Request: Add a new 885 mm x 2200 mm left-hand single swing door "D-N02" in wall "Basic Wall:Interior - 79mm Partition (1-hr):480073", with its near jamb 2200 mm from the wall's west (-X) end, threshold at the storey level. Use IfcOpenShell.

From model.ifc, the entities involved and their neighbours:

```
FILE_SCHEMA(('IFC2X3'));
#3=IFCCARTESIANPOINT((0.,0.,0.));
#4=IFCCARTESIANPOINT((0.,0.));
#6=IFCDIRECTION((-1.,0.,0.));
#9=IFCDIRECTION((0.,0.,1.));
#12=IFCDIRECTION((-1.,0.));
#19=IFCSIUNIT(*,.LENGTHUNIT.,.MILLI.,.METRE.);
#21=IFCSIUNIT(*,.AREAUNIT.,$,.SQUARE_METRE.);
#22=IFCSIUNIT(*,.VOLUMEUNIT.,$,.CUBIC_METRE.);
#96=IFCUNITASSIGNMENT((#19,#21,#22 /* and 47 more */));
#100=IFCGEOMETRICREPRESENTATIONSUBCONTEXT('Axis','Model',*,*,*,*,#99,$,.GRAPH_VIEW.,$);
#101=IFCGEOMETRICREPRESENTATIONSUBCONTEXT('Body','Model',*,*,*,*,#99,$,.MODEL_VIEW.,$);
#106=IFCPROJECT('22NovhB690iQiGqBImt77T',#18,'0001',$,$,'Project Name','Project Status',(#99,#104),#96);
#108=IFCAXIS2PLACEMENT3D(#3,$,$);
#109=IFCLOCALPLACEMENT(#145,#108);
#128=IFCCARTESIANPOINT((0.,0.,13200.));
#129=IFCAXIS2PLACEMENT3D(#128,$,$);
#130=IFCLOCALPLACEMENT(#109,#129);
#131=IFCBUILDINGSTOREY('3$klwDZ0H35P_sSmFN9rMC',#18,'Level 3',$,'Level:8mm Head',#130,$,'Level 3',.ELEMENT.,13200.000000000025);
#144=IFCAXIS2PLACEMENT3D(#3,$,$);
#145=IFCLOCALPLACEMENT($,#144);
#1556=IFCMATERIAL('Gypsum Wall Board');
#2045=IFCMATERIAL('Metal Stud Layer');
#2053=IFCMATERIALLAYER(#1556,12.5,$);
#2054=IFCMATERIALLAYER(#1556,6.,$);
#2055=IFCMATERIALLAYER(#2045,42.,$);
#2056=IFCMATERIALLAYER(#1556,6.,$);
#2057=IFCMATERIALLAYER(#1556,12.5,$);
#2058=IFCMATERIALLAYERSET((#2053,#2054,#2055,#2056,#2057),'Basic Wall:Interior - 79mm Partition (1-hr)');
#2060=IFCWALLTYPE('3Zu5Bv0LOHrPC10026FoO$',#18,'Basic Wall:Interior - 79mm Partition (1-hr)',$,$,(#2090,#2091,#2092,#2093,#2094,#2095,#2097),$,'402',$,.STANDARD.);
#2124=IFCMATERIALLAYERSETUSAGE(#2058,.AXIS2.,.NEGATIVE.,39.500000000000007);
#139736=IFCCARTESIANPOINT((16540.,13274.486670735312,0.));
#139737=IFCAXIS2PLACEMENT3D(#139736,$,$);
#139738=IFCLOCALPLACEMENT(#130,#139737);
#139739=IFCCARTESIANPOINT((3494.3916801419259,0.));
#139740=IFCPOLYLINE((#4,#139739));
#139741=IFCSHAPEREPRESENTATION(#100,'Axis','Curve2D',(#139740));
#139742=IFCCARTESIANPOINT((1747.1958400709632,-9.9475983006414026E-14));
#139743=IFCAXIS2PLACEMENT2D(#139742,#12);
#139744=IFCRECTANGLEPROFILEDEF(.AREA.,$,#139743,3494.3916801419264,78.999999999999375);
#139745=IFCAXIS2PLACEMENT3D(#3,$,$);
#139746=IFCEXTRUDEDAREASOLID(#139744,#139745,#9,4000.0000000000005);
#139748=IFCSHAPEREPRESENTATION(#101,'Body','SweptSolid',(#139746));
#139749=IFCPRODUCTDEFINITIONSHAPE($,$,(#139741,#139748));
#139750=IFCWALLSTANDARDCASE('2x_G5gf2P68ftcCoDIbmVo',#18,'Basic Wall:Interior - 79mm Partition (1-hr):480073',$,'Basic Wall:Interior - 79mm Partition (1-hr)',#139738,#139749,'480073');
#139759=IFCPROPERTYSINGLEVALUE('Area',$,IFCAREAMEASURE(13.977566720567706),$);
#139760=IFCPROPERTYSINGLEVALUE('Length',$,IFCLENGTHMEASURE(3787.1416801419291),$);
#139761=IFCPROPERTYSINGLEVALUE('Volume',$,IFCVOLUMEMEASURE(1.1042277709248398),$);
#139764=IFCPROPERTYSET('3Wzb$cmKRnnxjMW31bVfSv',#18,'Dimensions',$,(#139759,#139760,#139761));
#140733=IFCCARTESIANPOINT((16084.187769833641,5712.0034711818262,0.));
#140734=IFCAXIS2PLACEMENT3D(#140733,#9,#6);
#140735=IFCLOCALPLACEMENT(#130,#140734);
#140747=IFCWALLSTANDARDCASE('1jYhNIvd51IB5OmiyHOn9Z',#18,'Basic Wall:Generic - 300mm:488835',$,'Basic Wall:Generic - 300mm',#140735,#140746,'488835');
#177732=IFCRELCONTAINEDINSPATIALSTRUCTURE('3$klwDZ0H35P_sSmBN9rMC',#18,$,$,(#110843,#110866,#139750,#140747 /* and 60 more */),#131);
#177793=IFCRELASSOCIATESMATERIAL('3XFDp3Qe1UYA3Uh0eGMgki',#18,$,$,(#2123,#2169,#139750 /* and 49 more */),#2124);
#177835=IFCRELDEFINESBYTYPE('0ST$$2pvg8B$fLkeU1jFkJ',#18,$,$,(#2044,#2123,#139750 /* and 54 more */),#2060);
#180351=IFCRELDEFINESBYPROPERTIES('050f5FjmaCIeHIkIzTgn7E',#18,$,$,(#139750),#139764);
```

```python
import numpy as np
import ifcopenshell
import ifcopenshell.api.feature
import ifcopenshell.api.geometry
import ifcopenshell.api.pset
import ifcopenshell.api.root
import ifcopenshell.api.spatial
import ifcopenshell.api.type
import ifcopenshell.geom
import ifcopenshell.util.element
import ifcopenshell.util.placement
import ifcopenshell.util.representation
import ifcopenshell.util.shape
import ifcopenshell.util.unit

model = ifcopenshell.open("model.ifc")
unit_scale = ifcopenshell.util.unit.calculate_unit_scale(model)
area_scale = ifcopenshell.util.unit.calculate_unit_scale(model, "AREAUNIT")
volume_scale = ifcopenshell.util.unit.calculate_unit_scale(model, "VOLUMEUNIT")
settings = ifcopenshell.geom.settings()


def volume(element):
    """Net volume in cubic metres, openings subtracted."""
    shape = ifcopenshell.geom.create_shape(settings, element)
    return ifcopenshell.util.shape.get_volume(shape.geometry)


wall = model.by_id(139750)
storey = ifcopenshell.util.element.get_container(wall, ifc_class="IfcBuildingStorey")
context = ifcopenshell.util.representation.get_context(model, "Model", "Body", "MODEL_VIEW")
before = volume(wall)

width, height, from_end, sill = 0.885, 2.2, 2.2, 0.0  # metres

# The wall runs along its own X axis, and the end named is its -X end.
wall_shape = ifcopenshell.geom.create_shape(settings, wall)
x, y, z = ifcopenshell.util.shape.get_vertices(wall_shape.geometry).T
start = x.min() + from_end
face, thickness = float(y.min()), float(y.max() - y.min())
wall_matrix = ifcopenshell.util.placement.get_local_placement(wall.ObjectPlacement)
level = ifcopenshell.util.placement.get_local_placement(storey.ObjectPlacement)[2, 3]


def in_wall(x, y):
    """Placement at x, y metres in the wall's axes, at sill height."""
    matrix = wall_matrix.copy()
    matrix[:, 3] = wall_matrix @ np.array([x / unit_scale, y / unit_scale, 0.0, 1.0])
    matrix[2, 3] = level + sill / unit_scale
    return matrix


# Opening: a box that overshoots both wall faces by 50 mm.
opening = ifcopenshell.api.root.create_entity(model, ifc_class="IfcOpeningElement")
box = ifcopenshell.api.geometry.add_wall_representation(
    model, context=context, length=width, height=height, thickness=thickness + 0.1
)
ifcopenshell.api.geometry.assign_representation(model, product=opening, representation=box)
ifcopenshell.api.geometry.edit_object_placement(model, product=opening, matrix=in_wall(start, face - 0.05), is_si=False)
ifcopenshell.api.feature.add_feature(model, feature=opening, element=wall)

door = ifcopenshell.api.root.create_entity(model, ifc_class="IfcDoor", name="D-N02")
door.OverallWidth, door.OverallHeight = width / unit_scale, height / unit_scale
body = ifcopenshell.api.geometry.add_door_representation(
    model,
    context=context,
    overall_width=door.OverallWidth,
    overall_height=door.OverallHeight,
    operation_type="SINGLE_SWING_LEFT",
    lining_properties={"LiningDepth": thickness / unit_scale, "ThresholdDepth": thickness / unit_scale},
)
ifcopenshell.api.geometry.assign_representation(model, product=door, representation=body)
ifcopenshell.api.spatial.assign_container(model, products=[door], relating_structure=storey)
fills = ifcopenshell.api.feature.add_filling(model, opening=opening, element=door)
fills.OwnerHistory = door.OwnerHistory  # required in IFC2X3

# IFC2X3 keeps the operation on the door style.
style = ifcopenshell.api.root.create_entity(model, ifc_class="IfcDoorStyle", name="D-N02")
style.OperationType, style.ConstructionType = "SINGLE_SWING_LEFT", "NOTDEFINED"
style.ParameterTakesPrecedence = style.Sizeable = False
ifcopenshell.api.type.assign_type(model, related_objects=[door], relating_type=style)

# The lining spans the wall, so the door starts at the wall face.
ifcopenshell.api.geometry.edit_object_placement(model, product=door, matrix=in_wall(start, face), is_si=False)

after = volume(wall)

# Update the wall's stored quantities.
pset = model.by_id(ifcopenshell.util.element.get_pset(wall, "Dimensions", should_inherit=False)["id"])
ifcopenshell.api.pset.edit_pset(model, pset=pset, properties={
    "Area": model.create_entity("IfcAreaMeasure", after / thickness / area_scale),
    "Volume": model.create_entity("IfcVolumeMeasure", after / volume_scale),
})

print(f"wall volume {before:.3f} -> {after:.3f} m3")

model.write("model_edited.ifc")
```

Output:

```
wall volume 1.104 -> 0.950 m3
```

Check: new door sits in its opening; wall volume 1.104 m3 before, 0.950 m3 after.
